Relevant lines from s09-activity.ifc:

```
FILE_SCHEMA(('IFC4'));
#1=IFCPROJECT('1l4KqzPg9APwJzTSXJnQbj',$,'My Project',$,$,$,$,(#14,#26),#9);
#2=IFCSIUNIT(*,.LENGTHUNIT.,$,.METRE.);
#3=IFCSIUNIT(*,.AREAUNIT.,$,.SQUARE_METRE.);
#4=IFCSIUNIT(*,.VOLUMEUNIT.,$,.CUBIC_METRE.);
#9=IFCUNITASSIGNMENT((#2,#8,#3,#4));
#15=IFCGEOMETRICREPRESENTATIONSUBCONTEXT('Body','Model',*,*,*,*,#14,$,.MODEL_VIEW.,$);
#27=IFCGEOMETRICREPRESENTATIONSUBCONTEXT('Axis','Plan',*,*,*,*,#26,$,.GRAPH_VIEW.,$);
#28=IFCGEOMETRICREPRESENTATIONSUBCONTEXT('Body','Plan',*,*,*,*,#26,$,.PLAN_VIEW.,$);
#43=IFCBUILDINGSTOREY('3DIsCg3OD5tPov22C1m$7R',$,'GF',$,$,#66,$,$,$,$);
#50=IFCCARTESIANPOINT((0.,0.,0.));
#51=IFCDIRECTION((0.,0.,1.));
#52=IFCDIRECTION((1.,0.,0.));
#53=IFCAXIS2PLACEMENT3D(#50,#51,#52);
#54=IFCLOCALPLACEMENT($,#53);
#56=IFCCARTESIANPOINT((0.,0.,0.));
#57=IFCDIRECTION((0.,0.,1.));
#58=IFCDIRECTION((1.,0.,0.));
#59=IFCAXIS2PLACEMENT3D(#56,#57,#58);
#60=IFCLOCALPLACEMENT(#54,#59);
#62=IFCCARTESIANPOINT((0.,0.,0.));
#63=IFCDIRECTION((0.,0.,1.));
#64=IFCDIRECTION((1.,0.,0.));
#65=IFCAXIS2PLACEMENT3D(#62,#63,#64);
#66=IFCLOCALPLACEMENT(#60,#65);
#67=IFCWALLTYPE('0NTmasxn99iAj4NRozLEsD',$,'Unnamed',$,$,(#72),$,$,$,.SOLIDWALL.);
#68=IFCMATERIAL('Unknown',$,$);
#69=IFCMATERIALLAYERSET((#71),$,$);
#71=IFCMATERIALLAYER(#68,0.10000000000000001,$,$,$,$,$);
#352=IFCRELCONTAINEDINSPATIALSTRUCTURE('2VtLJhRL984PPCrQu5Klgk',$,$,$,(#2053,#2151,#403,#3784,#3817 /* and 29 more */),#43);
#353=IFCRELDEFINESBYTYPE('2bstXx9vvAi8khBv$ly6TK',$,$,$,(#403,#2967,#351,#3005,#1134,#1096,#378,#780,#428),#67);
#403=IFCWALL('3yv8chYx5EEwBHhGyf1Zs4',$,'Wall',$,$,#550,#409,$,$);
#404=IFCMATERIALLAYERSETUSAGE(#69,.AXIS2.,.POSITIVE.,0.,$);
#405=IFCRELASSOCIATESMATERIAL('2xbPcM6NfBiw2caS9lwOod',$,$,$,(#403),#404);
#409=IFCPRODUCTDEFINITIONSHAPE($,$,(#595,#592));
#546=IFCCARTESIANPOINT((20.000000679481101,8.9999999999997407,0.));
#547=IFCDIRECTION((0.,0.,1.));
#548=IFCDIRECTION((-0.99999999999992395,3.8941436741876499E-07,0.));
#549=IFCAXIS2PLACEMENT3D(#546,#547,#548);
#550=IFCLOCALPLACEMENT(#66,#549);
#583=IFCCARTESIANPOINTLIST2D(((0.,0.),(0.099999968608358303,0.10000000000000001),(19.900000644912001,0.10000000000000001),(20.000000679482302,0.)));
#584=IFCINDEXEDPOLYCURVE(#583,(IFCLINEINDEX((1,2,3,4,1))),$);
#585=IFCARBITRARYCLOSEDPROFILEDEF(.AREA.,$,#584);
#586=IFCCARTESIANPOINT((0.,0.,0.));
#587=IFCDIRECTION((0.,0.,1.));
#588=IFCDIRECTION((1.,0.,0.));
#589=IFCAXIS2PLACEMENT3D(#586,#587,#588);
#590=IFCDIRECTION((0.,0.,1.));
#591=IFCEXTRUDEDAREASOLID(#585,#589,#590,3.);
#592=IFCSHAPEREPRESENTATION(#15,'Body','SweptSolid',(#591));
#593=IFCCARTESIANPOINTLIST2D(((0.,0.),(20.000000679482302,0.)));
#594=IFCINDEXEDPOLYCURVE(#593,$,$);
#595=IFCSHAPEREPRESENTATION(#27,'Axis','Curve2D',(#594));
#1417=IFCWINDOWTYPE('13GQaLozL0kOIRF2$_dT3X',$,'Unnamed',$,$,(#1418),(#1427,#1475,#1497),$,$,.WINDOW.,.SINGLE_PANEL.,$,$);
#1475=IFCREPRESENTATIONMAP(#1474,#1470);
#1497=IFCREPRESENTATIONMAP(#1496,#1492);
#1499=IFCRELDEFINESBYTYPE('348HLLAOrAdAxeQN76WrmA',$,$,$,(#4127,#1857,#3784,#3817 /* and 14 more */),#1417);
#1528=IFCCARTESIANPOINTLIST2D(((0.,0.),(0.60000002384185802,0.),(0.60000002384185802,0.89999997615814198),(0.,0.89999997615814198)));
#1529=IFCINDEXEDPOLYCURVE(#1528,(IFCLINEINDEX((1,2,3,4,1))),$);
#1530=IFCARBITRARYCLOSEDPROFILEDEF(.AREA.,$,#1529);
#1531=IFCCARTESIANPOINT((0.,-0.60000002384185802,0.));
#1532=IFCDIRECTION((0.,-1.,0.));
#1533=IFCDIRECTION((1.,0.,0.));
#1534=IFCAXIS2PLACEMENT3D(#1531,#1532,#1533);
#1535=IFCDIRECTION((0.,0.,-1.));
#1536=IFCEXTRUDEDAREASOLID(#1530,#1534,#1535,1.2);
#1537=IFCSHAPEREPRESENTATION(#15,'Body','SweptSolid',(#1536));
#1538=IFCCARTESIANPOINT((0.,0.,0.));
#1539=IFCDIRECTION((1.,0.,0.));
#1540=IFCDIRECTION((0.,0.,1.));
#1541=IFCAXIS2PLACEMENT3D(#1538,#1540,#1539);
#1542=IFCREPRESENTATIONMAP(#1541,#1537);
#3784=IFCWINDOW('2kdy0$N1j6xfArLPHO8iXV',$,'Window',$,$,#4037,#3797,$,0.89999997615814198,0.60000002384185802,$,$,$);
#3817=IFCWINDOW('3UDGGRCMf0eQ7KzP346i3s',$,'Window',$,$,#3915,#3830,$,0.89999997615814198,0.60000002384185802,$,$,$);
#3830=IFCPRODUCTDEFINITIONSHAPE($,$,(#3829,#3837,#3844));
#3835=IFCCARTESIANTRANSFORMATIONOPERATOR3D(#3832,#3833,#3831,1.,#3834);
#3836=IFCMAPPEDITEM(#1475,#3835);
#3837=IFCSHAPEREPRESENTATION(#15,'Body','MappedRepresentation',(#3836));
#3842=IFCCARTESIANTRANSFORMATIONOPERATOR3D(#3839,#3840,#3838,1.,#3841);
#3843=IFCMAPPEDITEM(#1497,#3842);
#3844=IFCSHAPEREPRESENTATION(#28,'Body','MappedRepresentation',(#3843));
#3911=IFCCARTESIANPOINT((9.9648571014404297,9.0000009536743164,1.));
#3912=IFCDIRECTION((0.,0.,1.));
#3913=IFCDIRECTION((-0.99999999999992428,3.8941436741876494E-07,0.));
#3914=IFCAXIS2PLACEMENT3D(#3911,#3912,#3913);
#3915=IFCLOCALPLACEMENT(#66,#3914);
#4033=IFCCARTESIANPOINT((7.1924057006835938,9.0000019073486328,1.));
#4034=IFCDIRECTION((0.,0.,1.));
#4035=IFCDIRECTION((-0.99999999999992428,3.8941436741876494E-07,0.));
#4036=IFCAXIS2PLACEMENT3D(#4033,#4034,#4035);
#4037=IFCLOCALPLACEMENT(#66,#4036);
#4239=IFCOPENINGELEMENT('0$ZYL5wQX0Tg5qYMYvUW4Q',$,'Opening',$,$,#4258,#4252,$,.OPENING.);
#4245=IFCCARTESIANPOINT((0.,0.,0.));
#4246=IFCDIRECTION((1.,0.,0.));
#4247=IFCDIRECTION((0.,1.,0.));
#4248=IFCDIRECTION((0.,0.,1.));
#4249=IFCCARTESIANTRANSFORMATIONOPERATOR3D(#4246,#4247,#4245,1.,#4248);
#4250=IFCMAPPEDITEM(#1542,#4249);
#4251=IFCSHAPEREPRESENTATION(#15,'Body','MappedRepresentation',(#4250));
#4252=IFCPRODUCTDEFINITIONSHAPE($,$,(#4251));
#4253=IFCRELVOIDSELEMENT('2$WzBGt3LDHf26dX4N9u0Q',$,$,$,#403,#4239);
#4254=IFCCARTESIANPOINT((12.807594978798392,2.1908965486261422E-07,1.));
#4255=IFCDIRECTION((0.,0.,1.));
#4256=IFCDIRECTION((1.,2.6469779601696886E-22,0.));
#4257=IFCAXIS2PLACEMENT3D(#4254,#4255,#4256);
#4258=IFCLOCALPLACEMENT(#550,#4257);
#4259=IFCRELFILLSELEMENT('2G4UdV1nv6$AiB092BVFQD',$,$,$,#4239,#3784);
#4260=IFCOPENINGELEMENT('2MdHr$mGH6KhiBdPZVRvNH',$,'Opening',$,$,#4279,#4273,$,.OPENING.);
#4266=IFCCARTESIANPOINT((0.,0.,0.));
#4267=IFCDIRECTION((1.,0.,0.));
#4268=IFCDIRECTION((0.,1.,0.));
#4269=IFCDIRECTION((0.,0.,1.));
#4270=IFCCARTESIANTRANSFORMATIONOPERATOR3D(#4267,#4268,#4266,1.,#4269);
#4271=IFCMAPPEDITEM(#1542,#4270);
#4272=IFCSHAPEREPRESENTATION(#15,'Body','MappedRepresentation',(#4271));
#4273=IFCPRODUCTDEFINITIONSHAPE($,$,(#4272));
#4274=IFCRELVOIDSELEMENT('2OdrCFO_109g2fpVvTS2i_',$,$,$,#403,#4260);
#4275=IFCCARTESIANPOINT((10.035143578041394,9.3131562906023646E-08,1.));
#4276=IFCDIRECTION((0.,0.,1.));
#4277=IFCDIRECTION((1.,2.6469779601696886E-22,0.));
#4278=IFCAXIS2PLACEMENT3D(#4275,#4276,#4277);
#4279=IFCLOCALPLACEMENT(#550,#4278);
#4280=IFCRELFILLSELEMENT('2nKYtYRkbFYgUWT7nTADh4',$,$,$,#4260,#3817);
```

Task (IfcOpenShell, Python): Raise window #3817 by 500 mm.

```python
import numpy as np
import ifcopenshell
import ifcopenshell.api.geometry
import ifcopenshell.util.placement
import ifcopenshell.util.unit

model = ifcopenshell.open("s09-activity.ifc")
unit_scale = ifcopenshell.util.unit.calculate_unit_scale(model)

window = model.by_guid("3UDGGRCMf0eQ7KzP346i3s")
opening = window.FillsVoids[0].RelatingOpeningElement
dz = 0.5

shift = np.array([0.0, 0.0, dz])
# The window is not placed relative to its opening, so move both.
for product in (opening, window):
    matrix = ifcopenshell.util.placement.get_local_placement(product.ObjectPlacement)
    matrix[:3, 3] += shift
    ifcopenshell.api.geometry.edit_object_placement(model, product=product, matrix=matrix, is_si=False)

print(f"moved by {dz * unit_scale:+.3f} m")

model.write("s09-activity_rev.ifc")
```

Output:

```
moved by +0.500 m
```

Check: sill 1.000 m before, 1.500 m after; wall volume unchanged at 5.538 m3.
